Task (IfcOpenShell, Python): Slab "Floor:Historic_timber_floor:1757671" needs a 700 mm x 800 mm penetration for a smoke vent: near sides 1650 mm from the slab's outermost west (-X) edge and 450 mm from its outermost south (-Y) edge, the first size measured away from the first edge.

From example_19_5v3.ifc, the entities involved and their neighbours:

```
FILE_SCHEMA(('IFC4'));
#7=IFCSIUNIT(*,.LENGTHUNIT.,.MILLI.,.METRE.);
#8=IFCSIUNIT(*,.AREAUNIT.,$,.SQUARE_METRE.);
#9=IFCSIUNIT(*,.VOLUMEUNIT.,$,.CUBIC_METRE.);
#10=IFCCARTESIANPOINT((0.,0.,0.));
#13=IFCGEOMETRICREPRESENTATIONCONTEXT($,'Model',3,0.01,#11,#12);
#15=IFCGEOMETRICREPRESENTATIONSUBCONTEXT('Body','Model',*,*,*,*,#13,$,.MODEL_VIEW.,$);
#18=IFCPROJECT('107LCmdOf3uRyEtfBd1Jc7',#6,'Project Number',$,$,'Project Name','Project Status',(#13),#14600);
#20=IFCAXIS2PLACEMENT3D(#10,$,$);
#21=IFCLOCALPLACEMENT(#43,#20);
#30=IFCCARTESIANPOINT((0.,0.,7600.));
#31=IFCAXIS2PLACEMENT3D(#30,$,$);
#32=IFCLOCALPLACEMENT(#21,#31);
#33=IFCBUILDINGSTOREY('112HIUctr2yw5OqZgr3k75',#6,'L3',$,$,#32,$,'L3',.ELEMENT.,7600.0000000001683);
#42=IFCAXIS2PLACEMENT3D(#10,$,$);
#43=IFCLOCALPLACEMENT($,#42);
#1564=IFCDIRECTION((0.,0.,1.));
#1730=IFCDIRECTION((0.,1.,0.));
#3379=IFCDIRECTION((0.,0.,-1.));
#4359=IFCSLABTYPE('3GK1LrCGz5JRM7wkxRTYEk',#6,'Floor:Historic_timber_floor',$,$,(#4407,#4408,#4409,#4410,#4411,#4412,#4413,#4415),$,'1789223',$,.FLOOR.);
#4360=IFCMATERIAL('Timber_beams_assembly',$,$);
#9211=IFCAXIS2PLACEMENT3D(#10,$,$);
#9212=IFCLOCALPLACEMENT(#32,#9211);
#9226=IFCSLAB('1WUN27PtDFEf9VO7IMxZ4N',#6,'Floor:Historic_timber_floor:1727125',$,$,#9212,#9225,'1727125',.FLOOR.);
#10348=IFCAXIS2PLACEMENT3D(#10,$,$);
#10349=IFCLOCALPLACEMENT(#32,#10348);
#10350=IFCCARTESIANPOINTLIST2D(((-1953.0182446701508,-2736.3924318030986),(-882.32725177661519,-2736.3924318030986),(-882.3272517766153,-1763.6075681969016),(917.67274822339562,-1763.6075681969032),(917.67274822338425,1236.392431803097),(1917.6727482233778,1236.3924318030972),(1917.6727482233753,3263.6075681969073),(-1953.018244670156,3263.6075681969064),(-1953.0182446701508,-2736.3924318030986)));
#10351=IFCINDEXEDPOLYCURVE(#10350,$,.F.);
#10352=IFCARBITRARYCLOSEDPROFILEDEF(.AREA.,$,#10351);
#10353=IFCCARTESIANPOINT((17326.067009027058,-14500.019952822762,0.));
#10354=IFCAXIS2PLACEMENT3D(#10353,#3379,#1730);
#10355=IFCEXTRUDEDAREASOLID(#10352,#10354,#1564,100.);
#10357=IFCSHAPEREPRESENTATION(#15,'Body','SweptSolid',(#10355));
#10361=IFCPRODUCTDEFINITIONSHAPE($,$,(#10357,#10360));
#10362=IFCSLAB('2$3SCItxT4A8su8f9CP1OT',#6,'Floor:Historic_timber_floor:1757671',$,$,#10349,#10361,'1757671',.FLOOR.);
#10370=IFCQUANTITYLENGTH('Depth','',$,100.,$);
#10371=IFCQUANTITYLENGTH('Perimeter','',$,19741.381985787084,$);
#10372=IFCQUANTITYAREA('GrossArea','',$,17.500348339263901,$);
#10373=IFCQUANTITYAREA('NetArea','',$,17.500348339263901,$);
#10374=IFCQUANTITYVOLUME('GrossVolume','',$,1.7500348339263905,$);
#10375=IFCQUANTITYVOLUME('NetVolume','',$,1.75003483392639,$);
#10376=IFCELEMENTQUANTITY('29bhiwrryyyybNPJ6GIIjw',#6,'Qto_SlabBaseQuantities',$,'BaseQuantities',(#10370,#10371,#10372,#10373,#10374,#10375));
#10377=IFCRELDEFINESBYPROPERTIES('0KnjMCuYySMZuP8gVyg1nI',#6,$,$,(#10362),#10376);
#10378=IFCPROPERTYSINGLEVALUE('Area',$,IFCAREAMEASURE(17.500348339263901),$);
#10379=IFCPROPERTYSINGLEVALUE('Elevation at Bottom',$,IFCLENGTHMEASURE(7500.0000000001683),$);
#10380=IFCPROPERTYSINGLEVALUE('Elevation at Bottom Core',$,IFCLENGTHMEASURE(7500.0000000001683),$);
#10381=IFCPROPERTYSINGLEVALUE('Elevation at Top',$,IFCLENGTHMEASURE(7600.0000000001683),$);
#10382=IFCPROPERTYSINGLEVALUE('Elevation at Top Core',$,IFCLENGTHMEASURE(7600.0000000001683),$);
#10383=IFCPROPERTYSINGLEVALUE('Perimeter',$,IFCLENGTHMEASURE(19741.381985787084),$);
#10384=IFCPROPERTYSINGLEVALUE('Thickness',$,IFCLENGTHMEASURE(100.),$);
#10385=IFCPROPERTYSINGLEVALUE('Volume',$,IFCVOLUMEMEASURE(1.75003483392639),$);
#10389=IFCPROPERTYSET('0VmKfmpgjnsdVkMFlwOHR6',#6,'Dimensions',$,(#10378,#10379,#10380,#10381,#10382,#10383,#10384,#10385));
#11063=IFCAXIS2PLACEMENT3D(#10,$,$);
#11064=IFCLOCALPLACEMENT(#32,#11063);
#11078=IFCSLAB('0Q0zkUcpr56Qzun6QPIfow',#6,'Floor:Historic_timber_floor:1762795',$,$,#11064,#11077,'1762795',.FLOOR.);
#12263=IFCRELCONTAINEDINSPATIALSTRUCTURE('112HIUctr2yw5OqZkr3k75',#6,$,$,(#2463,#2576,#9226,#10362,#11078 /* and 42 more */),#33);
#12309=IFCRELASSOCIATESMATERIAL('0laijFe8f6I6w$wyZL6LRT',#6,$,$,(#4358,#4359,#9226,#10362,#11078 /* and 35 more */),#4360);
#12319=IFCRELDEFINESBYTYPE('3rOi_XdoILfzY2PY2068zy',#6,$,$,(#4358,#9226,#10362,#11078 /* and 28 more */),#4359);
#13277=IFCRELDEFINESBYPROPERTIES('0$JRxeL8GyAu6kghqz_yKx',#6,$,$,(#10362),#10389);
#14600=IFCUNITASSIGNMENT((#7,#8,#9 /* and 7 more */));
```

```python
import numpy as np
import ifcopenshell
import ifcopenshell.api.feature
import ifcopenshell.api.geometry
import ifcopenshell.api.pset
import ifcopenshell.api.root
import ifcopenshell.geom
import ifcopenshell.util.element
import ifcopenshell.util.placement
import ifcopenshell.util.representation
import ifcopenshell.util.shape
import ifcopenshell.util.unit

model = ifcopenshell.open("example_19_5v3.ifc")
unit_scale = ifcopenshell.util.unit.calculate_unit_scale(model)
area_scale = ifcopenshell.util.unit.calculate_unit_scale(model, "AREAUNIT")
volume_scale = ifcopenshell.util.unit.calculate_unit_scale(model, "VOLUMEUNIT")
settings = ifcopenshell.geom.settings()


def volume(element):
    """Net volume in cubic metres, openings subtracted."""
    shape = ifcopenshell.geom.create_shape(settings, element)
    return ifcopenshell.util.shape.get_volume(shape.geometry)


slab = model.by_id(10362)
before = volume(slab)

# Extent in the slab's own axes, in metres. The edges named are its -X and -Y sides.
slab_shape = ifcopenshell.geom.create_shape(settings, slab)
vertices = ifcopenshell.util.shape.get_vertices(slab_shape.geometry)
x_min, y_min, bottom = vertices.min(axis=0)
top = vertices[:, 2].max()

opening = ifcopenshell.api.root.create_entity(model, ifc_class="IfcOpeningElement", name="Smoke vent opening", predefined_type="OPENING")
context = ifcopenshell.util.representation.get_context(model, "Model", "Body", "MODEL_VIEW")
width, depth = 0.7, 0.8
outline = [(0.0, 0.0), (width, 0.0), (width, depth), (0.0, depth), (0.0, 0.0)]
# Overshoot both faces by 50 mm so the cut is clean.
shape = ifcopenshell.api.geometry.add_slab_representation(
    model, context=context, depth=top - bottom + 0.1, polyline=outline
)
ifcopenshell.api.geometry.assign_representation(model, product=opening, representation=shape)

matrix = ifcopenshell.util.placement.get_local_placement(slab.ObjectPlacement)
matrix[:, 3] = matrix @ np.append(np.array([x_min + 1.65, y_min + 0.45, bottom - 0.05]) / unit_scale, 1.0)
ifcopenshell.api.geometry.edit_object_placement(model, product=opening, matrix=matrix, is_si=False)
ifcopenshell.api.feature.add_feature(model, feature=opening, element=slab)

after = volume(slab)

# Update the slab's stored quantities.
qto = model.by_id(ifcopenshell.util.element.get_pset(slab, "Qto_SlabBaseQuantities", should_inherit=False)["id"])
ifcopenshell.api.pset.edit_qto(model, qto=qto, properties={
    "NetArea": after / (top - bottom) / area_scale,
    "NetVolume": after / volume_scale,
})
pset = model.by_id(ifcopenshell.util.element.get_pset(slab, "Dimensions", should_inherit=False)["id"])
ifcopenshell.api.pset.edit_pset(model, pset=pset, properties={
    "Area": model.create_entity("IfcAreaMeasure", after / (top - bottom) / area_scale),
    "Volume": model.create_entity("IfcVolumeMeasure", after / volume_scale),
})

print(f"slab volume {before:.3f} -> {after:.3f} m3")

model.write("example_19_5v3_updated.ifc")
```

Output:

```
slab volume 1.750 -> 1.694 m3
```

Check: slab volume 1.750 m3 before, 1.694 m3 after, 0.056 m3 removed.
